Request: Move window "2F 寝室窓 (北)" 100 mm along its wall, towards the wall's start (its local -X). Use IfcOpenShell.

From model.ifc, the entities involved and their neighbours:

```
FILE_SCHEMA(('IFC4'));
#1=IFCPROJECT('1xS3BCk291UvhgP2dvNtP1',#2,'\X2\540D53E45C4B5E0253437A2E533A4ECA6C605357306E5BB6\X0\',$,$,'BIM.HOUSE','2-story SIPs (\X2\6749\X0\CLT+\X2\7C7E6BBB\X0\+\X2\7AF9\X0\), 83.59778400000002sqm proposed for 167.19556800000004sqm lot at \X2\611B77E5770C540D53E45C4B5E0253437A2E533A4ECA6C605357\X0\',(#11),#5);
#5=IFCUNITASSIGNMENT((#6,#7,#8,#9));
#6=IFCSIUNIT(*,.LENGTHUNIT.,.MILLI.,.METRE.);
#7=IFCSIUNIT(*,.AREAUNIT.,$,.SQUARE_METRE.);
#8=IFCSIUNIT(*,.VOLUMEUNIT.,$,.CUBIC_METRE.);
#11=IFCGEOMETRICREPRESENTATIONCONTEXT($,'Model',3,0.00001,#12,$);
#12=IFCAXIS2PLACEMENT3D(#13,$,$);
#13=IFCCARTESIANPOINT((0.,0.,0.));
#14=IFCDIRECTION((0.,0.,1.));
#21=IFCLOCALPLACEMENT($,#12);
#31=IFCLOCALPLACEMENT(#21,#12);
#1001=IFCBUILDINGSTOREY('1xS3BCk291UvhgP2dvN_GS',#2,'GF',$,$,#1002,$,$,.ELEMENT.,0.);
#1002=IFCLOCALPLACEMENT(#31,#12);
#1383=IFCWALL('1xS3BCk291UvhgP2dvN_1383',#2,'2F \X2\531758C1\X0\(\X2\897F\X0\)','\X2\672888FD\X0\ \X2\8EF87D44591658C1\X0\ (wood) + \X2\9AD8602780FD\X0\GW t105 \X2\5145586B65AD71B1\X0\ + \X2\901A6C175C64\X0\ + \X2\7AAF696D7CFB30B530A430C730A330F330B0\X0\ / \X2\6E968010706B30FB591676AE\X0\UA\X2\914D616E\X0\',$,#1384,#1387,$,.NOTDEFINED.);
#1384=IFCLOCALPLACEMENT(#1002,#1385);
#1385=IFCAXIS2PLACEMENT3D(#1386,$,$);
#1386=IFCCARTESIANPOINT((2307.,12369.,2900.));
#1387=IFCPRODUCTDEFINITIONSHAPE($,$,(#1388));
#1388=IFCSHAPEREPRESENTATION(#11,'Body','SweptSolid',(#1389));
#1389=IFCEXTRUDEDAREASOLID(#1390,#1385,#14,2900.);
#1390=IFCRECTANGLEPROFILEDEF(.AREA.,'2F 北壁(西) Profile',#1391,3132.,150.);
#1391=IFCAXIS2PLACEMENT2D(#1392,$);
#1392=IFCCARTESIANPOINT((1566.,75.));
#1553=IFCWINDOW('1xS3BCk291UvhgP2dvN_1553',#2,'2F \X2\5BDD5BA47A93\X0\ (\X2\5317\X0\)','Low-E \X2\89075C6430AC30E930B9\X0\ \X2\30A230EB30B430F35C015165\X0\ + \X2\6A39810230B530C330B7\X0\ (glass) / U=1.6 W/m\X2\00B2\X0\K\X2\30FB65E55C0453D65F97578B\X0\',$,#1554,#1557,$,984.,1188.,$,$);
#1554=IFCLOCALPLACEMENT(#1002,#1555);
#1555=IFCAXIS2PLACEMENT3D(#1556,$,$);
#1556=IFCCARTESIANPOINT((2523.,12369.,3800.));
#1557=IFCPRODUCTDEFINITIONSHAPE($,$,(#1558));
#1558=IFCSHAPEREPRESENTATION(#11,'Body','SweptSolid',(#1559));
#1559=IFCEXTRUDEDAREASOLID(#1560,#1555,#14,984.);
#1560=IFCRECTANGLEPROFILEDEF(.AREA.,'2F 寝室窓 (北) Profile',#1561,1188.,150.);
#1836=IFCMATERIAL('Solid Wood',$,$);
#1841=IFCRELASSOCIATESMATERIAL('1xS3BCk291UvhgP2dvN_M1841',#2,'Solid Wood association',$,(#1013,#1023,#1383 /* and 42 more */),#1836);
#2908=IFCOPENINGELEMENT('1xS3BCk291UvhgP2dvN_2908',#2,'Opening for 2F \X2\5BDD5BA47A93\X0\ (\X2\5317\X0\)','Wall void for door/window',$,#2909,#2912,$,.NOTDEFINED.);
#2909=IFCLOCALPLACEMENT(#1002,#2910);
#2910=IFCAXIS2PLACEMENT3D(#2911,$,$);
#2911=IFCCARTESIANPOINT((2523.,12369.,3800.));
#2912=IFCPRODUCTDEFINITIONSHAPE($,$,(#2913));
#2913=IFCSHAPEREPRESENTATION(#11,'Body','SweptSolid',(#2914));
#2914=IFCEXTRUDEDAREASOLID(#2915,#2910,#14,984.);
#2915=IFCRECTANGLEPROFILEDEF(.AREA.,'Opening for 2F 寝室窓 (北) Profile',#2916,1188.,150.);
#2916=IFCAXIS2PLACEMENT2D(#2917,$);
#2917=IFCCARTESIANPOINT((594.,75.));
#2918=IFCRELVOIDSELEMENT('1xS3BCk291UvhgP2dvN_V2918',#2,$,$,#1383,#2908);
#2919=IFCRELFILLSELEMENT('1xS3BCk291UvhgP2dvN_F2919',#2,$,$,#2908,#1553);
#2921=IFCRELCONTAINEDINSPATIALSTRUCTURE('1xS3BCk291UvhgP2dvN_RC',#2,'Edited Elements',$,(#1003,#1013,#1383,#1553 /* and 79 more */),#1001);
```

```python
import ifcopenshell
import ifcopenshell.api.geometry
import ifcopenshell.util.placement
import ifcopenshell.util.unit

model = ifcopenshell.open("model.ifc")
unit_scale = ifcopenshell.util.unit.calculate_unit_scale(model)

window = model.by_guid("1xS3BCk291UvhgP2dvN_1553")
opening = window.FillsVoids[0].RelatingOpeningElement
wall = opening.VoidsElements[0].RelatingBuildingElement

wall_matrix = ifcopenshell.util.placement.get_local_placement(wall.ObjectPlacement)
shift = wall_matrix[:3, 0] * -0.1 / unit_scale
before = ifcopenshell.util.placement.get_local_placement(window.ObjectPlacement)[:3, 3].copy()

# The window is not placed relative to its opening, so move both.
for product in (opening, window):
    matrix = ifcopenshell.util.placement.get_local_placement(product.ObjectPlacement)
    matrix[:3, 3] += shift
    ifcopenshell.api.geometry.edit_object_placement(model, product=product, matrix=matrix, is_si=False)

after = ifcopenshell.util.placement.get_local_placement(window.ObjectPlacement)[:3, 3]
print("window moved by", (after - before).round(3) + 0.0)

model.write("model_v2.ifc")
```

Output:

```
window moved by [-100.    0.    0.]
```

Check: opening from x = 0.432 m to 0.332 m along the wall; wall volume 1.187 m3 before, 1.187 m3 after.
